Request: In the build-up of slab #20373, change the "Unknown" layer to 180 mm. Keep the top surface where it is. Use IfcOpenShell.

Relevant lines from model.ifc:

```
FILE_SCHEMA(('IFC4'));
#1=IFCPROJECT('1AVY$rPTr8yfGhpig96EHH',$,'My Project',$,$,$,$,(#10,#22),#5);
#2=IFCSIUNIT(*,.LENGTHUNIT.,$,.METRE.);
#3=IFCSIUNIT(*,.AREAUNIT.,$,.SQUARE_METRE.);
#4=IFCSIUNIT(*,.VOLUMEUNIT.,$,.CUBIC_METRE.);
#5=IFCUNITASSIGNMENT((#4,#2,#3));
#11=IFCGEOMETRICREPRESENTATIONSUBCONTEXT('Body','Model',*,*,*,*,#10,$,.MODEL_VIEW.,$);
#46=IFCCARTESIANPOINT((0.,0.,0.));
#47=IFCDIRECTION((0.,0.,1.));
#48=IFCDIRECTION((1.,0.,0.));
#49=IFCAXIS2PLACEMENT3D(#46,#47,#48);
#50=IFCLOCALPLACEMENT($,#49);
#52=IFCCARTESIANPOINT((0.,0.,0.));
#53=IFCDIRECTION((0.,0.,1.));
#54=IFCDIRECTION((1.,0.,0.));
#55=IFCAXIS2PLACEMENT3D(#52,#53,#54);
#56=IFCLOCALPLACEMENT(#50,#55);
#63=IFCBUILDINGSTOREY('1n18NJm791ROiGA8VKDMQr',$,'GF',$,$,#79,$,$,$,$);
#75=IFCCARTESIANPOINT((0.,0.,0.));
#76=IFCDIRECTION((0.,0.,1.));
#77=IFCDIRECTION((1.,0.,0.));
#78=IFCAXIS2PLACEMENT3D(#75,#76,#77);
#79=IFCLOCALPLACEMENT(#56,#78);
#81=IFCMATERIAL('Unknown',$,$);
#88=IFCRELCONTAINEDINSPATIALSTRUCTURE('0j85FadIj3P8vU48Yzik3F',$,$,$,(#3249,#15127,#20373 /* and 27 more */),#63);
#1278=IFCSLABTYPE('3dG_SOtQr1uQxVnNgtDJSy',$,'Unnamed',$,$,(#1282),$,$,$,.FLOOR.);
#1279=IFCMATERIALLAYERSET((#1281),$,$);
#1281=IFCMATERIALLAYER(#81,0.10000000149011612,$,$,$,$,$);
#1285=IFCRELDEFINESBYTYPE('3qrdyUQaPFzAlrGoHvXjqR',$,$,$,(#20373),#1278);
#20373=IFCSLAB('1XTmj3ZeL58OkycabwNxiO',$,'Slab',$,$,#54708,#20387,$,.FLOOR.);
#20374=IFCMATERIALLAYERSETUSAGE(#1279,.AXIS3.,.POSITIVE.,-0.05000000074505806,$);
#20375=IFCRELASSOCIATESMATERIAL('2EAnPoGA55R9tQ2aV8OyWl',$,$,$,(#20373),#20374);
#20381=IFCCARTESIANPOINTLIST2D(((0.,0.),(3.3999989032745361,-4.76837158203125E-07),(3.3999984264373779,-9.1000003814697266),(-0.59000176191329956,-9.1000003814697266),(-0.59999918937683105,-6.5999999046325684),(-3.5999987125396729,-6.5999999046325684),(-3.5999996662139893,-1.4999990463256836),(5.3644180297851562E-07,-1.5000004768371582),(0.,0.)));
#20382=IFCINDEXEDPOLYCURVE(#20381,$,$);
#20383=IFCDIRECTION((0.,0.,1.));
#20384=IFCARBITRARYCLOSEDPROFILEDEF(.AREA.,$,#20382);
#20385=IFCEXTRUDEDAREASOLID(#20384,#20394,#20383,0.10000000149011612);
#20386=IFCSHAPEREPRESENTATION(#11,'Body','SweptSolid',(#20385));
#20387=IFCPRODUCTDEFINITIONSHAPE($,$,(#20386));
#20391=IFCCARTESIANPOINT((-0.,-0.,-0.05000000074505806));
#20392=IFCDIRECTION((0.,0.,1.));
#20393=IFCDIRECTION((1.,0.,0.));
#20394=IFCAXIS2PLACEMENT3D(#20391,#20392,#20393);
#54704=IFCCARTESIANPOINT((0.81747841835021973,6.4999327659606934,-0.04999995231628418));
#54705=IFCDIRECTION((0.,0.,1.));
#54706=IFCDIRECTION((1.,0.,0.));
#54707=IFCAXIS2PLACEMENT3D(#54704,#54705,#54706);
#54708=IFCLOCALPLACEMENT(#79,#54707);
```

```python
import ifcopenshell
import ifcopenshell.util.element
import ifcopenshell.util.representation
import ifcopenshell.util.unit

model = ifcopenshell.open("model.ifc")
unit_scale = ifcopenshell.util.unit.calculate_unit_scale(model)

layer_set = model.by_id(1279)
layer = next(l for l in layer_set.MaterialLayers if l.Material and l.Material.Name == "Unknown")
change = 0.18 / unit_scale - layer.LayerThickness
layer.LayerThickness += change

# Geometry does not follow the layer set by itself.
slabs = [e for e in ifcopenshell.util.element.get_elements_by_material(model, layer_set) if e.is_a("IfcSlab")]
for slab in sorted(slabs, key=lambda e: e.id()):
    body = ifcopenshell.util.representation.get_representation(slab, "Model", "Body")
    solid = body.Items[0]
    old_depth = solid.Depth
    solid.Depth += change
    # Extruded upwards: lower the start of the extrusion so the top stays.
    x, y, z = solid.Position.Location.Coordinates
    solid.Position.Location = model.createIfcCartesianPoint((x, y, z - change))
    print(slab.id(), f"{old_depth:g} -> {solid.Depth:g}")

# The layers are counted up from the underside, which has moved.
for usage in {ifcopenshell.util.element.get_material(slab) for slab in slabs}:
    usage.OffsetFromReferenceLine -= change

model.write("model_edited.ifc")
```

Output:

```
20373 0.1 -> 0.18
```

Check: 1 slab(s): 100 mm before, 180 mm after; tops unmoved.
